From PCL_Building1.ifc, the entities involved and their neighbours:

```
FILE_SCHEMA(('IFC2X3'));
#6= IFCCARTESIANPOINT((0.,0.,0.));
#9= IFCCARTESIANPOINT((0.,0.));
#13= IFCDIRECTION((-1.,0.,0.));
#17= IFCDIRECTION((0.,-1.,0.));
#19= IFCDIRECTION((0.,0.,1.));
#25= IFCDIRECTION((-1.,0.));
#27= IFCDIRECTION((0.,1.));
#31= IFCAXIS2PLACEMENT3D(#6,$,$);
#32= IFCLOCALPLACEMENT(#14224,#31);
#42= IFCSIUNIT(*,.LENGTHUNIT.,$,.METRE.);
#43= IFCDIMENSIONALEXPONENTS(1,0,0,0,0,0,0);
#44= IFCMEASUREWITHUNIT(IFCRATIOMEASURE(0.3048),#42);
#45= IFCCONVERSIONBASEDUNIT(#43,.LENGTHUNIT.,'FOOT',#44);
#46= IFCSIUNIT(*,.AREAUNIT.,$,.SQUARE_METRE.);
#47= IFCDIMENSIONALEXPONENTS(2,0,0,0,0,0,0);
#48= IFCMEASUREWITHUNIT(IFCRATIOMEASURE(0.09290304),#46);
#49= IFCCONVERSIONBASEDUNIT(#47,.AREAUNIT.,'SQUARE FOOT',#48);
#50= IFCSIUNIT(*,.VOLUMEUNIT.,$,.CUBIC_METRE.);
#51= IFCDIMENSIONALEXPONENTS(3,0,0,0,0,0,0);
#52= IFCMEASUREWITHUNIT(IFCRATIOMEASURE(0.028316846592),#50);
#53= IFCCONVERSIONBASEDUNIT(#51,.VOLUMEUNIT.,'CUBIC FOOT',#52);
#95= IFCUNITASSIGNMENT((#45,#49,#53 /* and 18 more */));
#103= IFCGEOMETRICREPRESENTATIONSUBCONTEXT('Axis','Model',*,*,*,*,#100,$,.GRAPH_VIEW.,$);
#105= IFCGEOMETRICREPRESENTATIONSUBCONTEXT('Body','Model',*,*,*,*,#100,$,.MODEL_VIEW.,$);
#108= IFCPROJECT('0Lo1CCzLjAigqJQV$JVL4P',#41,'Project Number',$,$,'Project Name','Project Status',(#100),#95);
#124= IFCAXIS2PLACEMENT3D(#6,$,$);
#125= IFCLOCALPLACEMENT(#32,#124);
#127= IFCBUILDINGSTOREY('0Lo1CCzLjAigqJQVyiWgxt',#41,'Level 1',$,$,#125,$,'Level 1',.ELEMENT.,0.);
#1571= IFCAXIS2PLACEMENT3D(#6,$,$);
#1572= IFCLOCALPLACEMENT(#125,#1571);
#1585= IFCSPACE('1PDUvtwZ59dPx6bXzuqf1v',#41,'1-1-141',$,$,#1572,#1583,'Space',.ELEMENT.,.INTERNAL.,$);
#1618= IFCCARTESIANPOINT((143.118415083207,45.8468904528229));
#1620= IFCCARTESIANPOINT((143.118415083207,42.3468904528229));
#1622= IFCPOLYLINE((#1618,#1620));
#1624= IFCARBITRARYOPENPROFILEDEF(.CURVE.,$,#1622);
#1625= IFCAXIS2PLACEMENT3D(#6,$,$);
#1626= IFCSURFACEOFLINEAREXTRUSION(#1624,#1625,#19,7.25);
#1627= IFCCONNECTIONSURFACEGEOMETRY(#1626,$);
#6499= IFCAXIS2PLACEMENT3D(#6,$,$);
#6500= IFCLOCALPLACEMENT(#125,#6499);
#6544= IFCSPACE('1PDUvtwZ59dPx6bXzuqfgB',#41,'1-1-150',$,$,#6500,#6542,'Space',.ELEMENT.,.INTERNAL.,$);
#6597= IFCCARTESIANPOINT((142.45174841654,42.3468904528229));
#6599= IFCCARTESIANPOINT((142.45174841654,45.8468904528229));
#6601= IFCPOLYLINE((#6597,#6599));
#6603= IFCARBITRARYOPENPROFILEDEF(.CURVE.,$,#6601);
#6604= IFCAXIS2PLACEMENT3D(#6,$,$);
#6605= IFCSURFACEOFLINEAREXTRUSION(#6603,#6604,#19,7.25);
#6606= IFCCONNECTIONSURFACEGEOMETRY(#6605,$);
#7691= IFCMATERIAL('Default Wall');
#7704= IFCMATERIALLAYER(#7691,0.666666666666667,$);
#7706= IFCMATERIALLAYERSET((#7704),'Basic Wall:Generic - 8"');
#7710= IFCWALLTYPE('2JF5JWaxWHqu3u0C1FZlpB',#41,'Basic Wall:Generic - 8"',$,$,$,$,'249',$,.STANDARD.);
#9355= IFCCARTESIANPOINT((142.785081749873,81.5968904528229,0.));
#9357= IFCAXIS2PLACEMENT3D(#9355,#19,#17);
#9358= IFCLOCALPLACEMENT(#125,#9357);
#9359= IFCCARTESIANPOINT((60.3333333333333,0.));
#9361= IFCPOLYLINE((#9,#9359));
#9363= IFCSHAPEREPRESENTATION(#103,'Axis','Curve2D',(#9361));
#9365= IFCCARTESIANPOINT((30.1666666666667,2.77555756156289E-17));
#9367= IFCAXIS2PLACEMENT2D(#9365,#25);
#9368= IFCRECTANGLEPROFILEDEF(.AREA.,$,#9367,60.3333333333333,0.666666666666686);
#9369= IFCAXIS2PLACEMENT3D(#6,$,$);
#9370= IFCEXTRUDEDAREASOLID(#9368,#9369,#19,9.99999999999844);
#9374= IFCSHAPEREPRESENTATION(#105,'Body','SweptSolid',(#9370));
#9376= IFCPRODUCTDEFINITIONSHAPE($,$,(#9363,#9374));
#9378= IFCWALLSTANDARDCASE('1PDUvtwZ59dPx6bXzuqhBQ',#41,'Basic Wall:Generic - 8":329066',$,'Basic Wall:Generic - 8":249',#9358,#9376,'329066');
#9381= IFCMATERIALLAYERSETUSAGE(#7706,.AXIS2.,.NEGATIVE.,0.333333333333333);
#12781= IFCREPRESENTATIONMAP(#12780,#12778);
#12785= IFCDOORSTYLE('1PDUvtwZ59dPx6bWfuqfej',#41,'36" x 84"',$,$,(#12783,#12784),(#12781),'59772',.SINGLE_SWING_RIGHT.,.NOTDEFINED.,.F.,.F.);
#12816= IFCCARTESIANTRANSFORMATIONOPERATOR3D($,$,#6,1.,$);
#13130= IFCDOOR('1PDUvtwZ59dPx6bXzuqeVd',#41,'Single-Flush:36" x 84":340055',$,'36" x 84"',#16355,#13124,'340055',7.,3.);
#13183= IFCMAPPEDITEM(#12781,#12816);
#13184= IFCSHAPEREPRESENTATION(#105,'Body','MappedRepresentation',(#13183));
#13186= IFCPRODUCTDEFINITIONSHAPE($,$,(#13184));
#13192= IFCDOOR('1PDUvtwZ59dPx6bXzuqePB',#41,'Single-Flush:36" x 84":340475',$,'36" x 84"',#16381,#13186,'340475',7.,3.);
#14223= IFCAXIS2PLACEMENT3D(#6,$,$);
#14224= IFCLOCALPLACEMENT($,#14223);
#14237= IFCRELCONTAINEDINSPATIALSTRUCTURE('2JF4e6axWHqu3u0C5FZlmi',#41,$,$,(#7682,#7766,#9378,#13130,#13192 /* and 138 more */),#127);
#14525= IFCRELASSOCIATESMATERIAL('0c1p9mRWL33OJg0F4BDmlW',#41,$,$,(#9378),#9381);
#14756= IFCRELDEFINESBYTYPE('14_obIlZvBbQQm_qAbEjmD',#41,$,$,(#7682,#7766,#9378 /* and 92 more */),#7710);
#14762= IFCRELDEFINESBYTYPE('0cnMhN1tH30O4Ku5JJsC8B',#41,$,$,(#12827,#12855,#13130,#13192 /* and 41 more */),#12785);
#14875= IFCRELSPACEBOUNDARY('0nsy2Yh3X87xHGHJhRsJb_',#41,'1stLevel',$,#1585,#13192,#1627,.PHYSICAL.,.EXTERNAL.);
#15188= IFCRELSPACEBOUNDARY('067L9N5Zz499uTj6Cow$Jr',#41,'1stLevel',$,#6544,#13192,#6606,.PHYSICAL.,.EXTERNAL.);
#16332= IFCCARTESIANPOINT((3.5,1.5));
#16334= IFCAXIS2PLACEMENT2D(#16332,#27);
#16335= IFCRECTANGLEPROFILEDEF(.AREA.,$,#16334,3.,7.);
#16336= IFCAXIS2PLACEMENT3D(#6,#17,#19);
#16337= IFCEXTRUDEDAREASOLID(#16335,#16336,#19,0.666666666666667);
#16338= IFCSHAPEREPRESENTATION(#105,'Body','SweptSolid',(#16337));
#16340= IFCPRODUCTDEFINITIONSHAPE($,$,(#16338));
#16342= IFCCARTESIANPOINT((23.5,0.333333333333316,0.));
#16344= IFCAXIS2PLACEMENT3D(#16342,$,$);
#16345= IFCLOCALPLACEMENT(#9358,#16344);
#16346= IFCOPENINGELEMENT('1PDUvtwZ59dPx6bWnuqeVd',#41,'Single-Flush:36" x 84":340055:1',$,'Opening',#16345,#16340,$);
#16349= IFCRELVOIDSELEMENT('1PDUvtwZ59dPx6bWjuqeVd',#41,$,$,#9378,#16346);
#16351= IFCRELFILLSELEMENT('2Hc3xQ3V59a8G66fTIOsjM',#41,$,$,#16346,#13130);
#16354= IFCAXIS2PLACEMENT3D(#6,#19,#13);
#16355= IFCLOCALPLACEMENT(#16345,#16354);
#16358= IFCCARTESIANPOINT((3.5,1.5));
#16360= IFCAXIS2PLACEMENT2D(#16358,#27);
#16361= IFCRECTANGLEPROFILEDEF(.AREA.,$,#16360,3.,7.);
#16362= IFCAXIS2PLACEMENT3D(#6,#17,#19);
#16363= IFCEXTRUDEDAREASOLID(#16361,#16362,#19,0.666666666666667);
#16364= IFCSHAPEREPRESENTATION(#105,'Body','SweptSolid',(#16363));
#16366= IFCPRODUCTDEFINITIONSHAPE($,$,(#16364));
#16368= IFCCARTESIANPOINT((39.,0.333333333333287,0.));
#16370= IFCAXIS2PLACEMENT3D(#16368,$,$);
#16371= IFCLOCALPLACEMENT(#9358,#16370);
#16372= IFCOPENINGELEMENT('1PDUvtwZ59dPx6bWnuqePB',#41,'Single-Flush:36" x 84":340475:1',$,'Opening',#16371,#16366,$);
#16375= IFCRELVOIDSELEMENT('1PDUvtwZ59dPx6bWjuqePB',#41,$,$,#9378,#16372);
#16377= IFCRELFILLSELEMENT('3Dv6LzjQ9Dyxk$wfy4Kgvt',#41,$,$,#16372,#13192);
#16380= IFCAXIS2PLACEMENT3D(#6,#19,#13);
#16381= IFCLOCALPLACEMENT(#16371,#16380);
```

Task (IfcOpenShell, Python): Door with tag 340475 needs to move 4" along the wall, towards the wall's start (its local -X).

```python
import numpy as np
import ifcopenshell
import ifcopenshell.api.geometry
import ifcopenshell.util.placement
import ifcopenshell.util.unit

model = ifcopenshell.open("PCL_Building1.ifc")
unit_scale = ifcopenshell.util.unit.calculate_unit_scale(model)

door = model.by_guid("1PDUvtwZ59dPx6bXzuqePB")
opening = door.FillsVoids[0].RelatingOpeningElement
wall = opening.VoidsElements[0].RelatingBuildingElement

wall_matrix = ifcopenshell.util.placement.get_local_placement(wall.ObjectPlacement)
shift = wall_matrix[:3, 0] * -4 * 0.0254 / unit_scale
before = ifcopenshell.util.placement.get_local_placement(door.ObjectPlacement)[:3, 3].copy()

# The door is placed relative to its opening, so it follows when the opening moves.
matrix = ifcopenshell.util.placement.get_local_placement(opening.ObjectPlacement)
matrix[:3, 3] += shift
ifcopenshell.api.geometry.edit_object_placement(
    model, product=opening, matrix=matrix, is_si=False, should_transform_children=True
)

# Space boundary surfaces are stored in each space's coordinates; move them too.
for rel in door.ProvidesBoundaries:
    if not rel.ConnectionGeometry:
        continue
    surface = rel.ConnectionGeometry.SurfaceOnRelatingElement
    space_matrix = ifcopenshell.util.placement.get_local_placement(rel.RelatingSpace.ObjectPlacement)
    point = np.array(surface.Position.Location.Coordinates) + space_matrix[:3, :3].T @ shift
    surface.Position = model.createIfcAxis2Placement3D(
        model.createIfcCartesianPoint(point.tolist()), surface.Position.Axis, surface.Position.RefDirection
    )

after = ifcopenshell.util.placement.get_local_placement(door.ObjectPlacement)[:3, 3]
print("door moved by", (after - before).round(3) + 0.0)

model.write("PCL_Building1_rev.ifc")
```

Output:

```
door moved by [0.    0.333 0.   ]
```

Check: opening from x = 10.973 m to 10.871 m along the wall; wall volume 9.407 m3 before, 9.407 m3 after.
